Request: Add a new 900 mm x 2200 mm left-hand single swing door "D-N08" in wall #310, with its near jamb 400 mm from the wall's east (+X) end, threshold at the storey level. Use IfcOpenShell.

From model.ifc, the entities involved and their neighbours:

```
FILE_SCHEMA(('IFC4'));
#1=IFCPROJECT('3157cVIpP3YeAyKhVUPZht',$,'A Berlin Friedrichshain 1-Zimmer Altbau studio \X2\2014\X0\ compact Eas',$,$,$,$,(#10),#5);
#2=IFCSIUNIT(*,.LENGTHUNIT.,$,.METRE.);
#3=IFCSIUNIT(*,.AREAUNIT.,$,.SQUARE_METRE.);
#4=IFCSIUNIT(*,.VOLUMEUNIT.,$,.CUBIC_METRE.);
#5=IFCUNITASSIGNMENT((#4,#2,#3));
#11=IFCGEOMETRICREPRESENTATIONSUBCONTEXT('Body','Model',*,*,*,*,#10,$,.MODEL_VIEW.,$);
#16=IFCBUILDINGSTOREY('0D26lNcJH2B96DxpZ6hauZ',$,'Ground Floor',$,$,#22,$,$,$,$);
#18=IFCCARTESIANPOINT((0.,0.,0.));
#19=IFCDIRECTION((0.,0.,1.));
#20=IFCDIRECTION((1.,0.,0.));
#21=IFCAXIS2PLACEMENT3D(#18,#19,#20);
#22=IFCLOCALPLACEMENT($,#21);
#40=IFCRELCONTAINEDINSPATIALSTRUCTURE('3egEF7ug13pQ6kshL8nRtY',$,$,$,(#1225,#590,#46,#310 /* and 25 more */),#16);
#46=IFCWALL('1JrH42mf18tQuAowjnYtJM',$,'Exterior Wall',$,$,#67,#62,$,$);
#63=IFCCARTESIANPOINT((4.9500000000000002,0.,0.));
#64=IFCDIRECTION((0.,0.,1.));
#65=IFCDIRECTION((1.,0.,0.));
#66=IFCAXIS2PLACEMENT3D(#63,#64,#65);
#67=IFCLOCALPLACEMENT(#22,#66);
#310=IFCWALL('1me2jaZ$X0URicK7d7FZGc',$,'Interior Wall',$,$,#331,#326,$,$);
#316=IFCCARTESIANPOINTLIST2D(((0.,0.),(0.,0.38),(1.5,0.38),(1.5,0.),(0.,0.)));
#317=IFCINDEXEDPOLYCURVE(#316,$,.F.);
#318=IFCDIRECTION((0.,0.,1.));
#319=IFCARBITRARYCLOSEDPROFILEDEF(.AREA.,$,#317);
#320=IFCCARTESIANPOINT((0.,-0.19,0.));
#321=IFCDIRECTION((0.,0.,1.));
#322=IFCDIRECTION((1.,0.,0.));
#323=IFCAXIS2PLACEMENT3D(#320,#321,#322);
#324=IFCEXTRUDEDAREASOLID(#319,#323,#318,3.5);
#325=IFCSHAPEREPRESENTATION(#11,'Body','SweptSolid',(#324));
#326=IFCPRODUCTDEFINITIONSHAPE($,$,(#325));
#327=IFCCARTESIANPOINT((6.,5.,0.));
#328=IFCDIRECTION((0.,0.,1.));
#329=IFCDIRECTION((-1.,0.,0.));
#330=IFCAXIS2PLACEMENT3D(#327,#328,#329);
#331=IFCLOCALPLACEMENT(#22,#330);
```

```python
import numpy as np
import ifcopenshell
import ifcopenshell.api.feature
import ifcopenshell.api.geometry
import ifcopenshell.api.root
import ifcopenshell.api.spatial
import ifcopenshell.geom
import ifcopenshell.util.element
import ifcopenshell.util.placement
import ifcopenshell.util.representation
import ifcopenshell.util.shape
import ifcopenshell.util.unit

model = ifcopenshell.open("model.ifc")
unit_scale = ifcopenshell.util.unit.calculate_unit_scale(model)
settings = ifcopenshell.geom.settings()


def volume(element):
    """Net volume in cubic metres, openings subtracted."""
    shape = ifcopenshell.geom.create_shape(settings, element)
    return ifcopenshell.util.shape.get_volume(shape.geometry)


wall = model.by_guid("1me2jaZ$X0URicK7d7FZGc")
storey = ifcopenshell.util.element.get_container(wall, ifc_class="IfcBuildingStorey")
context = ifcopenshell.util.representation.get_context(model, "Model", "Body", "MODEL_VIEW")
before = volume(wall)

width, height, from_end, sill = 0.9, 2.2, 0.4, 0.0  # metres

# The wall runs along its own X axis, and the end named is its -X end.
wall_shape = ifcopenshell.geom.create_shape(settings, wall)
x, y, z = ifcopenshell.util.shape.get_vertices(wall_shape.geometry).T
start = x.min() + from_end
face, thickness = float(y.min()), float(y.max() - y.min())
wall_matrix = ifcopenshell.util.placement.get_local_placement(wall.ObjectPlacement)
level = ifcopenshell.util.placement.get_local_placement(storey.ObjectPlacement)[2, 3]


def in_wall(x, y):
    """Placement at x, y metres in the wall's axes, at sill height."""
    matrix = wall_matrix.copy()
    matrix[:, 3] = wall_matrix @ np.array([x / unit_scale, y / unit_scale, 0.0, 1.0])
    matrix[2, 3] = level + sill / unit_scale
    return matrix


# Opening: a box that overshoots both wall faces by 50 mm.
opening = ifcopenshell.api.root.create_entity(model, ifc_class="IfcOpeningElement", predefined_type="OPENING")
box = ifcopenshell.api.geometry.add_wall_representation(
    model, context=context, length=width, height=height, thickness=thickness + 0.1
)
ifcopenshell.api.geometry.assign_representation(model, product=opening, representation=box)
ifcopenshell.api.geometry.edit_object_placement(model, product=opening, matrix=in_wall(start, face - 0.05), is_si=False)
ifcopenshell.api.feature.add_feature(model, feature=opening, element=wall)

door = ifcopenshell.api.root.create_entity(model, ifc_class="IfcDoor", name="D-N08", predefined_type="DOOR")
door.OverallWidth, door.OverallHeight = width / unit_scale, height / unit_scale
door.OperationType = "SINGLE_SWING_LEFT"
body = ifcopenshell.api.geometry.add_door_representation(
    model,
    context=context,
    overall_width=door.OverallWidth,
    overall_height=door.OverallHeight,
    operation_type="SINGLE_SWING_LEFT",
    lining_properties={"LiningDepth": thickness / unit_scale, "ThresholdDepth": thickness / unit_scale},
)
ifcopenshell.api.geometry.assign_representation(model, product=door, representation=body)
ifcopenshell.api.spatial.assign_container(model, products=[door], relating_structure=storey)
ifcopenshell.api.feature.add_filling(model, opening=opening, element=door)

# The lining spans the wall, so the door starts at the wall face.
ifcopenshell.api.geometry.edit_object_placement(model, product=door, matrix=in_wall(start, face), is_si=False)

after = volume(wall)

print(f"wall volume {before:.3f} -> {after:.3f} m3")

model.write("model_rev.ifc")
```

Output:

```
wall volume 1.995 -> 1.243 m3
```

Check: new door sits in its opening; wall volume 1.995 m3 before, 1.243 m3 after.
